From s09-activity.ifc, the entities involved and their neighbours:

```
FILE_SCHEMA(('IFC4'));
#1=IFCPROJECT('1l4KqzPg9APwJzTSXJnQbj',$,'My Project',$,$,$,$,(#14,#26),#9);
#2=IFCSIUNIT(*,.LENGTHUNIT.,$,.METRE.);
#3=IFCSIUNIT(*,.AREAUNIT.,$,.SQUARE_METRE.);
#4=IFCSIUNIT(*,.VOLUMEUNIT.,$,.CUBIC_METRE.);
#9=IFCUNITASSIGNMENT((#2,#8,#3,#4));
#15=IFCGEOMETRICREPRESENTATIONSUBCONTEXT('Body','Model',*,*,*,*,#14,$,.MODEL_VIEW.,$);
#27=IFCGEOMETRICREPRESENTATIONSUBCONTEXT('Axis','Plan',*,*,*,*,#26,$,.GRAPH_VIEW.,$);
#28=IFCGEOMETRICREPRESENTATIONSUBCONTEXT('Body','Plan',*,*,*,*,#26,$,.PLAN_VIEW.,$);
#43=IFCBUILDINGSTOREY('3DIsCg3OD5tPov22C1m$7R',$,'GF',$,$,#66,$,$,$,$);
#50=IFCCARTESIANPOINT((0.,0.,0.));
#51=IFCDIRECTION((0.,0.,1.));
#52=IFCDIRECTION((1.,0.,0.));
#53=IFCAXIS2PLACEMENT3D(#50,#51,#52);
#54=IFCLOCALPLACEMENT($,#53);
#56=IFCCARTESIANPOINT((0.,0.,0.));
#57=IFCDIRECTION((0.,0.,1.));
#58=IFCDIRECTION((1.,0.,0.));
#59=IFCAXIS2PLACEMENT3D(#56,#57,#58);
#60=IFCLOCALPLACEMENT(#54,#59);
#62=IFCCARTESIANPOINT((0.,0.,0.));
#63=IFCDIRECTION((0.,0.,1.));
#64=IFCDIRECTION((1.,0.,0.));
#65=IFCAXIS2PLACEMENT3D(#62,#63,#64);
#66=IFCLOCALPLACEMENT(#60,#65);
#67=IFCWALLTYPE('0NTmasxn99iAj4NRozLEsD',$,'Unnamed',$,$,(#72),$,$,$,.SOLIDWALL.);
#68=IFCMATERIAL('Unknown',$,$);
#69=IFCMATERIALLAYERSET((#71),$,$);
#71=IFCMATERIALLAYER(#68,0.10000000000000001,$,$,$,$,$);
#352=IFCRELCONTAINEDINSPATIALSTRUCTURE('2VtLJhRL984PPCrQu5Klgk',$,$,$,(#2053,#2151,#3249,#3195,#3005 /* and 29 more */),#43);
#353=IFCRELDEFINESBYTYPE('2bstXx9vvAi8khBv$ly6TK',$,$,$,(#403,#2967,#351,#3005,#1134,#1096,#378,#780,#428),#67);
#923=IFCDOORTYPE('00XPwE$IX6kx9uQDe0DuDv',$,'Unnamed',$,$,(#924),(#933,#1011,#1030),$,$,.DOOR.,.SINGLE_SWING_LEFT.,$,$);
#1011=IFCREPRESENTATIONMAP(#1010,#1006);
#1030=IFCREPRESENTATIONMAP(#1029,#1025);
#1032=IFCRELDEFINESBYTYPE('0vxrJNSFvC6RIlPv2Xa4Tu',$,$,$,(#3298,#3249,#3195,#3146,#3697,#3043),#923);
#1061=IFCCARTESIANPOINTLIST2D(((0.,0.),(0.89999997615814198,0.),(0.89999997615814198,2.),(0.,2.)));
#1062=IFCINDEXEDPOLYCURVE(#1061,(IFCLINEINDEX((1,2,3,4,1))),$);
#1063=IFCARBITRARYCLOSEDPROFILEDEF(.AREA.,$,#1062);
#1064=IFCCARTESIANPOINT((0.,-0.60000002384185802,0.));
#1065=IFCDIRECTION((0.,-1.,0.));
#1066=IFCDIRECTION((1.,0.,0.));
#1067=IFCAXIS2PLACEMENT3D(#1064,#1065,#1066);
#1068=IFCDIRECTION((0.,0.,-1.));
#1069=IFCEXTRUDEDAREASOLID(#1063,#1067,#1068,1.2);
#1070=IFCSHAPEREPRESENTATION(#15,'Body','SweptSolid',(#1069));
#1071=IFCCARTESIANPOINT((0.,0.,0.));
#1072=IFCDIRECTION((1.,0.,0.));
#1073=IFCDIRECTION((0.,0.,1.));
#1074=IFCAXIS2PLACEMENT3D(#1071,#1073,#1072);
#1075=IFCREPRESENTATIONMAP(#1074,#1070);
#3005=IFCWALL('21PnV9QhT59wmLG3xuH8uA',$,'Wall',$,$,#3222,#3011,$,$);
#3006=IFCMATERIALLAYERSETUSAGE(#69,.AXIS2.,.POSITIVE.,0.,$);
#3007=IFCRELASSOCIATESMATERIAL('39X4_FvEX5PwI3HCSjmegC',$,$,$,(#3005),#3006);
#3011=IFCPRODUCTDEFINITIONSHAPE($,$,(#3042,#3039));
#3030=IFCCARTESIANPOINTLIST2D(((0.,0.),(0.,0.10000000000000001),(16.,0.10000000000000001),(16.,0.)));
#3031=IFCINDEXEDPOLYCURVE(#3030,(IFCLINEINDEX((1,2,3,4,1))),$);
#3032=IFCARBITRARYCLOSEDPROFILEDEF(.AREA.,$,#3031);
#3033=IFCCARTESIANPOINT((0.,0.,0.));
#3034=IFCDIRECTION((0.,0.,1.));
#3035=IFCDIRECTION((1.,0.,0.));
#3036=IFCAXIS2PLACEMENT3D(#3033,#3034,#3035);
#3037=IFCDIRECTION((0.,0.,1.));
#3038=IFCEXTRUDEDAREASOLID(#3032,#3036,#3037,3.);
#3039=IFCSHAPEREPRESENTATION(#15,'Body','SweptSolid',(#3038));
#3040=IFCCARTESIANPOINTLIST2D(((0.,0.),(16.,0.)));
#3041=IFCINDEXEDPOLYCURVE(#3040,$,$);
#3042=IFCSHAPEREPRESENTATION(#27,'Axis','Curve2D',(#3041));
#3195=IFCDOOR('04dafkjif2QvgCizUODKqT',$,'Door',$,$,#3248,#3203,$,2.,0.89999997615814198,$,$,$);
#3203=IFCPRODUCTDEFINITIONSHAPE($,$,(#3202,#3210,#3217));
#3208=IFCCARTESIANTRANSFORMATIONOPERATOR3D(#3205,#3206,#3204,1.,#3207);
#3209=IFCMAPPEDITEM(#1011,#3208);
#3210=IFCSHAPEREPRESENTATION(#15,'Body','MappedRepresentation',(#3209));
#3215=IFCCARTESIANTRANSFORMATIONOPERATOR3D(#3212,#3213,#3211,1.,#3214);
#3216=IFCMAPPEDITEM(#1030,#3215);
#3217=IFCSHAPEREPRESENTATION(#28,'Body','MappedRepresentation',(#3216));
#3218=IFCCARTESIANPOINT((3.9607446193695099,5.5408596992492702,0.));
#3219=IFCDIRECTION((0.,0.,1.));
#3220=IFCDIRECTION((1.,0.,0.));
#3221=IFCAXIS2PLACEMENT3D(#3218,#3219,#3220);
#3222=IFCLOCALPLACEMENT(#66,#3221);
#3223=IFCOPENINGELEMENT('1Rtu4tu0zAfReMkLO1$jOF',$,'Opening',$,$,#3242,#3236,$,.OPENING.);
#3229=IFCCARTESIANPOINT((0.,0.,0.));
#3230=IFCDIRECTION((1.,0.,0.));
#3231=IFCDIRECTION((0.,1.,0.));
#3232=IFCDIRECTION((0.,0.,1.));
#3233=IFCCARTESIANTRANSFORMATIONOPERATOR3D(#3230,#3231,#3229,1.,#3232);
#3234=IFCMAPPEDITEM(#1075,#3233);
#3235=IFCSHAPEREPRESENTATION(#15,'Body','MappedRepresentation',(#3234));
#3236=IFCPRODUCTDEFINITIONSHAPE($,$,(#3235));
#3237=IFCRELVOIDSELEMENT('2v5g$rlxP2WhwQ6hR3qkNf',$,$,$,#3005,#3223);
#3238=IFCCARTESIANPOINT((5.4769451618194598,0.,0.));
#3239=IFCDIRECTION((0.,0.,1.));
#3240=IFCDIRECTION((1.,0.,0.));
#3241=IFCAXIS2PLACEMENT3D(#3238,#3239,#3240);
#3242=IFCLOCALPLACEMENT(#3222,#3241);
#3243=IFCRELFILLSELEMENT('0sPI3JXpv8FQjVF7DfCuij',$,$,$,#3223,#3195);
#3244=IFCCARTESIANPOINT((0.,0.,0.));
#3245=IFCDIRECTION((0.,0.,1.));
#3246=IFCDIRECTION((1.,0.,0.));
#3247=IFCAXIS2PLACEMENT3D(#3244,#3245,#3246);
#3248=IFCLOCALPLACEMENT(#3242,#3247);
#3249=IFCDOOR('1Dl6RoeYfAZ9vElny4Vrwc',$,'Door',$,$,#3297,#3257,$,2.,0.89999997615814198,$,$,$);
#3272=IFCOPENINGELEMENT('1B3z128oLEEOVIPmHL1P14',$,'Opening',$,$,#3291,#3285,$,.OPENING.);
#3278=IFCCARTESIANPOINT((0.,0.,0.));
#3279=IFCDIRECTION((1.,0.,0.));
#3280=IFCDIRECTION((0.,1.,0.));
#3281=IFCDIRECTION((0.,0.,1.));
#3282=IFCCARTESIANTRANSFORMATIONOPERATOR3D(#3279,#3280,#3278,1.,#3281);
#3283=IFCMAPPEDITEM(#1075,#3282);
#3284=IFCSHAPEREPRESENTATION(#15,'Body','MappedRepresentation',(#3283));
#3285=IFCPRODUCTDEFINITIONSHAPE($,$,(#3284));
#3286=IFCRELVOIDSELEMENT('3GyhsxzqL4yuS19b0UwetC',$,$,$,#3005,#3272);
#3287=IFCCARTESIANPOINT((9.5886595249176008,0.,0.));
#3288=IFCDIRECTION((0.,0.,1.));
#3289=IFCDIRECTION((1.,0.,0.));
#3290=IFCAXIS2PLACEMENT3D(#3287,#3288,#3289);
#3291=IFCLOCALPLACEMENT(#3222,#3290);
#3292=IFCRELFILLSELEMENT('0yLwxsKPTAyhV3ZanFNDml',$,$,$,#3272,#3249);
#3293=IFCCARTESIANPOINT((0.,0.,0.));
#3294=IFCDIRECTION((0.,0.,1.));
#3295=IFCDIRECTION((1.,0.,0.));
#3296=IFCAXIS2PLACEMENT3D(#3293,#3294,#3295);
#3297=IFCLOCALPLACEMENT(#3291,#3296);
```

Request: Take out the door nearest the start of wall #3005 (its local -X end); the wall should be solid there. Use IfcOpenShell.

```python
import ifcopenshell
import ifcopenshell.api.feature
import ifcopenshell.api.root
import ifcopenshell.geom
import ifcopenshell.util.shape

model = ifcopenshell.open("s09-activity.ifc")
settings = ifcopenshell.geom.settings()


def volume(element):
    """Net volume in cubic metres, openings subtracted."""
    shape = ifcopenshell.geom.create_shape(settings, element)
    return ifcopenshell.util.shape.get_volume(shape.geometry)


door = model.by_guid("04dafkjif2QvgCizUODKqT")
opening = door.FillsVoids[0].RelatingOpeningElement
wall = opening.VoidsElements[0].RelatingBuildingElement
before = volume(wall)

ifcopenshell.api.root.remove_product(model, product=door)
ifcopenshell.api.feature.remove_feature(model, feature=opening)

after = volume(wall)

print(f"wall volume {before:.3f} -> {after:.3f} m3")

model.write("s09-activity_updated.ifc")
```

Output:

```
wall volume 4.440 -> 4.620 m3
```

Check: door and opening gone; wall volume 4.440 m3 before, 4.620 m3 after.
